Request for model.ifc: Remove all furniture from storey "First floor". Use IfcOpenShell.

First a look at what the model holds.

```python
import ifcopenshell
import ifcopenshell.util.element

model = ifcopenshell.open("model.ifc")
print(model.schema)
storey = next(s for s in model.by_type("IfcBuildingStorey") if s.Name == "First floor")
furniture = [e for e in ifcopenshell.util.element.get_decomposition(storey) if e.is_a("IfcFurnishingElement")]
seen = {}
for e in furniture:
    element_type = ifcopenshell.util.element.get_type(e)
    name = element_type.Name if element_type not in (None, e) else None
    seen[name] = seen.get(name, 0) + 1
for name, count in sorted(seen.items(), key=str):
    print(count, "x", name)
```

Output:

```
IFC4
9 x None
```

```python
import ifcopenshell
import ifcopenshell.api.root
import ifcopenshell.util.element

model = ifcopenshell.open("model.ifc")

storey = next(s for s in model.by_type("IfcBuildingStorey") if s.Name == "First floor")
furniture = [e for e in ifcopenshell.util.element.get_decomposition(storey) if e.is_a("IfcFurnishingElement")]

for e in furniture:
    ifcopenshell.api.root.remove_product(model, product=e)
print(len(furniture), "removed")

model.write("model_rev.ifc")
```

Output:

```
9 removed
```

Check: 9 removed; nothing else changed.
